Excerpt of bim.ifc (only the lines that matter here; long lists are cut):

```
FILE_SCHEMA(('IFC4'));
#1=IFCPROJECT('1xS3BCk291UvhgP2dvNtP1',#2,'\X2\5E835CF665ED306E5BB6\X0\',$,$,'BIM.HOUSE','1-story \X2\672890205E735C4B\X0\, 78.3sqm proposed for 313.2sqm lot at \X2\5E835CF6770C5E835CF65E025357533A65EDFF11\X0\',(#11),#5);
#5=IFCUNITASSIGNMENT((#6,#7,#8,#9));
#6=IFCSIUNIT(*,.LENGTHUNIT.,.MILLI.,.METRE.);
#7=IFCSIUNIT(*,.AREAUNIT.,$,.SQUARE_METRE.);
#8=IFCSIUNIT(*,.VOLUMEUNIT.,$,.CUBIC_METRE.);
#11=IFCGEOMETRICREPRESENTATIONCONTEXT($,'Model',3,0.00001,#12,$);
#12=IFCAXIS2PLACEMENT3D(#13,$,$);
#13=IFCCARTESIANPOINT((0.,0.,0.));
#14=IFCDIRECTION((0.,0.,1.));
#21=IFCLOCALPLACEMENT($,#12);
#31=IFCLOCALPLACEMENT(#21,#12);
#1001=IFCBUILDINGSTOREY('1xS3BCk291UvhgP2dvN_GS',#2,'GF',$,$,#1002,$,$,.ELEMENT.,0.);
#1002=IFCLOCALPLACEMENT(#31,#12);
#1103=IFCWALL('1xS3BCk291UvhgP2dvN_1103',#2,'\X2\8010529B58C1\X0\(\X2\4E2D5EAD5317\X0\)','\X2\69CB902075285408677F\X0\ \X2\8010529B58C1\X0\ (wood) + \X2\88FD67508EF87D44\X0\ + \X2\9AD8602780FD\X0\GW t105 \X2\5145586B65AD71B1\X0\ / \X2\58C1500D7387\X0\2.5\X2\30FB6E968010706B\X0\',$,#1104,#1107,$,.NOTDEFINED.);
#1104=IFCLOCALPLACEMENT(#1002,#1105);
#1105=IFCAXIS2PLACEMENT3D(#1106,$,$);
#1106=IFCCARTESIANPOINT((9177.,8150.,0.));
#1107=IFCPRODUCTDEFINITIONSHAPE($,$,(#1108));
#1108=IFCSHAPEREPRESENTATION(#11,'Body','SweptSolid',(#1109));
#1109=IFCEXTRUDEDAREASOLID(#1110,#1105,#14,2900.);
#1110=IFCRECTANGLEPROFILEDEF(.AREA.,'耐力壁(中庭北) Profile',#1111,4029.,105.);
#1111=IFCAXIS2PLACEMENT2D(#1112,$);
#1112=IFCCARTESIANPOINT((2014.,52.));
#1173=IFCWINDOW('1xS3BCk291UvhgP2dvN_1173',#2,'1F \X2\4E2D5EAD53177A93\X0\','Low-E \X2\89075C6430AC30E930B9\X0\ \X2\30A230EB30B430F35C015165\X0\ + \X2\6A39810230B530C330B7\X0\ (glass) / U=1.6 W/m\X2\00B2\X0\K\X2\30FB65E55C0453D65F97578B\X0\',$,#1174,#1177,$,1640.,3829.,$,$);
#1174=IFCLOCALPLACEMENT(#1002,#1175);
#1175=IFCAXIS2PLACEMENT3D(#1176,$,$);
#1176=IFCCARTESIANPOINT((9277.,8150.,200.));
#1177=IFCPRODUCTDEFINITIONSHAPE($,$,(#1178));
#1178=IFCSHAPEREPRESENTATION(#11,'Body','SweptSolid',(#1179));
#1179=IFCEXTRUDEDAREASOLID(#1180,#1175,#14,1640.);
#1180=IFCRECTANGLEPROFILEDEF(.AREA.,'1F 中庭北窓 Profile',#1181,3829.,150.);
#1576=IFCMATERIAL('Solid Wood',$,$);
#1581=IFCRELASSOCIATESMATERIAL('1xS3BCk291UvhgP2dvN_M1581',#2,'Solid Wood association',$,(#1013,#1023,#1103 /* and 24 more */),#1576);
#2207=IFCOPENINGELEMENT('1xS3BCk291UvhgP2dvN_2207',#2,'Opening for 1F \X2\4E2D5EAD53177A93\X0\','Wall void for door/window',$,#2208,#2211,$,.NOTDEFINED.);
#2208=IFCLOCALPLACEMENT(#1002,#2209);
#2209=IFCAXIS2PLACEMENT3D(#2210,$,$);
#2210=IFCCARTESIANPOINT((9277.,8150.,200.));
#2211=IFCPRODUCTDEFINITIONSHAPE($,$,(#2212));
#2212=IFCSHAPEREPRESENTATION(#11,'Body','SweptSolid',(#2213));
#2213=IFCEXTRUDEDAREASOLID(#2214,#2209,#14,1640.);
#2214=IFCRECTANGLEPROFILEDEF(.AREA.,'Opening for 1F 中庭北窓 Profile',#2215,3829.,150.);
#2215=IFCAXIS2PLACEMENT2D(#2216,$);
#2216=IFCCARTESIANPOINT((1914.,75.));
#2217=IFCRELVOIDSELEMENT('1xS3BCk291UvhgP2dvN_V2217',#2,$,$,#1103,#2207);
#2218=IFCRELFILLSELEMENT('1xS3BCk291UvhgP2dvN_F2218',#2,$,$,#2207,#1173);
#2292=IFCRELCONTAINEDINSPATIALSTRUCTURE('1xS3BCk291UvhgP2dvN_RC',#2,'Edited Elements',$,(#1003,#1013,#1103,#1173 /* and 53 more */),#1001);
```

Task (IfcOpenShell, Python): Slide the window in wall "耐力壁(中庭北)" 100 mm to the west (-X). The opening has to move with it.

```python
import ifcopenshell
import ifcopenshell.api.geometry
import ifcopenshell.util.placement

model = ifcopenshell.open("bim.ifc")

window = model.by_guid("1xS3BCk291UvhgP2dvN_1173")
opening = window.FillsVoids[0].RelatingOpeningElement
wall = opening.VoidsElements[0].RelatingBuildingElement

wall_matrix = ifcopenshell.util.placement.get_local_placement(wall.ObjectPlacement)
shift = wall_matrix[:3, 0] * -100.0
before = ifcopenshell.util.placement.get_local_placement(window.ObjectPlacement)[:3, 3].copy()

# The window is not placed relative to its opening, so move both.
for product in (opening, window):
    matrix = ifcopenshell.util.placement.get_local_placement(product.ObjectPlacement)
    matrix[:3, 3] += shift
    ifcopenshell.api.geometry.edit_object_placement(model, product=product, matrix=matrix, is_si=False)

after = ifcopenshell.util.placement.get_local_placement(window.ObjectPlacement)[:3, 3]
print("window moved by", (after - before).round(3) + 0.0)

model.write("bim-out.ifc")
```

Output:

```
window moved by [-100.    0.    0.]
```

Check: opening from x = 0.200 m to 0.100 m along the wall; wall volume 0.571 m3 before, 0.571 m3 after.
